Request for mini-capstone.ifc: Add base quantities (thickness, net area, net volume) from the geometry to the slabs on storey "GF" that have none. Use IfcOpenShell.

First a look at what the model holds.

```python
import ifcopenshell
import ifcopenshell.util.element
import ifcopenshell.util.unit

model = ifcopenshell.open("mini-capstone.ifc")
print(model.schema)
for unit_type in ("LENGTHUNIT", "AREAUNIT", "VOLUMEUNIT"):
    print(unit_type, ifcopenshell.util.unit.calculate_unit_scale(model, unit_type))
storey = next(s for s in model.by_type("IfcBuildingStorey") if s.Name == "GF")
slabs = [e for e in ifcopenshell.util.element.get_decomposition(storey) if e.is_a("IfcSlab")]
for e in sorted(slabs, key=lambda e: e.id()):
    print(e.id(), e.is_a(), e.Name, list(ifcopenshell.util.element.get_psets(e, qtos_only=True)), sep=" | ")
```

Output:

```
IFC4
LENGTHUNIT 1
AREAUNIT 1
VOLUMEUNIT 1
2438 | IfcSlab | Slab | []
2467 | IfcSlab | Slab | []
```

```python
import ifcopenshell
import ifcopenshell.api.pset
import ifcopenshell.geom
import ifcopenshell.util.element
import ifcopenshell.util.shape
import ifcopenshell.util.unit

model = ifcopenshell.open("mini-capstone.ifc")
unit_scale = ifcopenshell.util.unit.calculate_unit_scale(model)
area_scale = ifcopenshell.util.unit.calculate_unit_scale(model, "AREAUNIT")
volume_scale = ifcopenshell.util.unit.calculate_unit_scale(model, "VOLUMEUNIT")
settings = ifcopenshell.geom.settings()

storey = next(s for s in model.by_type("IfcBuildingStorey") if s.Name == "GF")
slabs = [e for e in ifcopenshell.util.element.get_decomposition(storey) if e.is_a("IfcSlab")]

for e in sorted(slabs, key=lambda e: e.id()):
    if ifcopenshell.util.element.get_psets(e, qtos_only=True, should_inherit=False):
        continue
    # Geometry comes back in metres, in the element's own axes.
    shape = ifcopenshell.geom.create_shape(settings, e)
    values = {
        "Width": ifcopenshell.util.shape.get_z(shape.geometry) / unit_scale,
        "NetArea": ifcopenshell.util.shape.get_footprint_area(shape.geometry) / area_scale,
        "NetVolume": ifcopenshell.util.shape.get_volume(shape.geometry) / volume_scale,
    }
    qto = ifcopenshell.api.pset.add_qto(model, product=e, name="Qto_SlabBaseQuantities")
    ifcopenshell.api.pset.edit_qto(model, qto=qto, properties=values)
    print(e.id(), {k: round(v, 3) for k, v in values.items()})

model.write("mini-capstone-out.ifc")
```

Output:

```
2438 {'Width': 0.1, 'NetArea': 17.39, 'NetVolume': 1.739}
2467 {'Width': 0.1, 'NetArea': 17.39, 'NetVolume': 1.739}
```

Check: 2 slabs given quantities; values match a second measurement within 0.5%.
